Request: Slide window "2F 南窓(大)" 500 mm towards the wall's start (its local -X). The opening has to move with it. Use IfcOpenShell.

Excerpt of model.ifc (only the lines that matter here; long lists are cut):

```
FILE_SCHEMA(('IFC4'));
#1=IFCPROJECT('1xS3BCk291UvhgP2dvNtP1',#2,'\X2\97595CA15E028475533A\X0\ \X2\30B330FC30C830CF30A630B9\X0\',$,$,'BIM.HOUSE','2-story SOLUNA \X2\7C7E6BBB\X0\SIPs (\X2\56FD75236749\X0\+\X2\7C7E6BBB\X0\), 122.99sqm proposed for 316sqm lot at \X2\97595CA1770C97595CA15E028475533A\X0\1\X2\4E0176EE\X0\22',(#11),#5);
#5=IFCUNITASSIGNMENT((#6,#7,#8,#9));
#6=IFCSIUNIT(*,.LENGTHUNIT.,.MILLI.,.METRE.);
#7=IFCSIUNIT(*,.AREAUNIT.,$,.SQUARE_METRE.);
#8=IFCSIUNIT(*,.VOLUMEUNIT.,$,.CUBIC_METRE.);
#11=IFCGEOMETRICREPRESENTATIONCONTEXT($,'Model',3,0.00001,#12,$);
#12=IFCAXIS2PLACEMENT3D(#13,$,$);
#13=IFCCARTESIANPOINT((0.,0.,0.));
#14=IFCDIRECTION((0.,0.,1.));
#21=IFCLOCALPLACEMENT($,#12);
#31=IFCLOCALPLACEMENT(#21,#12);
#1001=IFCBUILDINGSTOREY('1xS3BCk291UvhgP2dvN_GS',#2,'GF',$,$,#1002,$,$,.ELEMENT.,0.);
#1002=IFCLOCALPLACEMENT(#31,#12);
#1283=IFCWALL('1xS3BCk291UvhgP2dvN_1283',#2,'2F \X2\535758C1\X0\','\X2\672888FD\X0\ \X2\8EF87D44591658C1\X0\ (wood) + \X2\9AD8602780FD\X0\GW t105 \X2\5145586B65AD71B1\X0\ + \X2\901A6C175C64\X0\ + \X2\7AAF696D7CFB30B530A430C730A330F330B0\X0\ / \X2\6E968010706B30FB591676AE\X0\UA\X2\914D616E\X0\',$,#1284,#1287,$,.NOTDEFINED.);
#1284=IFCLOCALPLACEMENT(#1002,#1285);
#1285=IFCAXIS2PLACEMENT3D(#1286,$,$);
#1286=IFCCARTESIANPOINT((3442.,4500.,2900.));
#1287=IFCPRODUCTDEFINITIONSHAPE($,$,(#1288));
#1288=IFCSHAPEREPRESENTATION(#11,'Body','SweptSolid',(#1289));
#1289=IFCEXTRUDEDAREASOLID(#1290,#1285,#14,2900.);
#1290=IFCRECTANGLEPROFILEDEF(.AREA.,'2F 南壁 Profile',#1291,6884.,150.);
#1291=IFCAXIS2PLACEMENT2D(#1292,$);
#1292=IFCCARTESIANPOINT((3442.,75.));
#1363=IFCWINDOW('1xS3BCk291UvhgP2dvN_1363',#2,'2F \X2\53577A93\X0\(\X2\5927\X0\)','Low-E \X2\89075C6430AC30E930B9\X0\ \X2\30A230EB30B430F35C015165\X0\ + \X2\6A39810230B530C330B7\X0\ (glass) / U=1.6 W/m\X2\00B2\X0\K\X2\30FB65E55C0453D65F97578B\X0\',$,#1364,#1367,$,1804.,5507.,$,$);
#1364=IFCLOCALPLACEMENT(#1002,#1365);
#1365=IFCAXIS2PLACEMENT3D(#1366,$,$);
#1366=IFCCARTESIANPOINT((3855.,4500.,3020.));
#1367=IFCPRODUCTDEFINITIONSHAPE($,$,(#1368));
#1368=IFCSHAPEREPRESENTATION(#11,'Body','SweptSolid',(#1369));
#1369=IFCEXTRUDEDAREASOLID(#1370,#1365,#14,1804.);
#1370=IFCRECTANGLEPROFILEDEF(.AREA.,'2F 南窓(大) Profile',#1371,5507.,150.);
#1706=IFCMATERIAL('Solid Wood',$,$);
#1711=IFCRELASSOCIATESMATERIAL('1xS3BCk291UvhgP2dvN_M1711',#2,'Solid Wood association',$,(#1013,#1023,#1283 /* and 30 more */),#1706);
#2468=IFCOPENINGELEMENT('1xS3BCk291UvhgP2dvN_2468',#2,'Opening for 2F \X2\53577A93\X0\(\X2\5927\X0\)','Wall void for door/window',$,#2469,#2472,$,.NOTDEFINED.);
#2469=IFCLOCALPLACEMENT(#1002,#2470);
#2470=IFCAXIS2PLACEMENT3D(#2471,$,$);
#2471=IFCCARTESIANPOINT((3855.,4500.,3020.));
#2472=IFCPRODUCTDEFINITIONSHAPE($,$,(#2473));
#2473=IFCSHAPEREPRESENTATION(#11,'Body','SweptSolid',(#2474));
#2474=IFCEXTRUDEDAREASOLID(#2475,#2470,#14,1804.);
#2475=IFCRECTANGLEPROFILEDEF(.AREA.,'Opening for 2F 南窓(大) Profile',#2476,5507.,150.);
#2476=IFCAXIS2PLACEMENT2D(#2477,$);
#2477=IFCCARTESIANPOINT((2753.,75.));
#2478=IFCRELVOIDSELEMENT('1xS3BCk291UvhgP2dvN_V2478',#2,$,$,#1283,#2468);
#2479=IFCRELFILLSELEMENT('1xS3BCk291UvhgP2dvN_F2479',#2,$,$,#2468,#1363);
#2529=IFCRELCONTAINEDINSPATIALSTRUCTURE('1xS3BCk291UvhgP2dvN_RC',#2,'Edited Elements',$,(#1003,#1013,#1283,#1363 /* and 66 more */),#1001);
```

```python
import ifcopenshell
import ifcopenshell.api.geometry
import ifcopenshell.util.placement

model = ifcopenshell.open("model.ifc")

window = model.by_guid("1xS3BCk291UvhgP2dvN_1363")
opening = window.FillsVoids[0].RelatingOpeningElement
wall = opening.VoidsElements[0].RelatingBuildingElement

wall_matrix = ifcopenshell.util.placement.get_local_placement(wall.ObjectPlacement)
shift = wall_matrix[:3, 0] * -500.0
before = ifcopenshell.util.placement.get_local_placement(window.ObjectPlacement)[:3, 3].copy()

# The window is not placed relative to its opening, so move both.
for product in (opening, window):
    matrix = ifcopenshell.util.placement.get_local_placement(product.ObjectPlacement)
    matrix[:3, 3] += shift
    ifcopenshell.api.geometry.edit_object_placement(model, product=product, matrix=matrix, is_si=False)

after = ifcopenshell.util.placement.get_local_placement(window.ObjectPlacement)[:3, 3]
print("window moved by", (after - before).round(3) + 0.0)

model.write("model_edited.ifc")
```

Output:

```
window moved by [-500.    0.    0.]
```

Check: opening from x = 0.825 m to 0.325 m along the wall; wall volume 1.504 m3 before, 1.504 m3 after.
